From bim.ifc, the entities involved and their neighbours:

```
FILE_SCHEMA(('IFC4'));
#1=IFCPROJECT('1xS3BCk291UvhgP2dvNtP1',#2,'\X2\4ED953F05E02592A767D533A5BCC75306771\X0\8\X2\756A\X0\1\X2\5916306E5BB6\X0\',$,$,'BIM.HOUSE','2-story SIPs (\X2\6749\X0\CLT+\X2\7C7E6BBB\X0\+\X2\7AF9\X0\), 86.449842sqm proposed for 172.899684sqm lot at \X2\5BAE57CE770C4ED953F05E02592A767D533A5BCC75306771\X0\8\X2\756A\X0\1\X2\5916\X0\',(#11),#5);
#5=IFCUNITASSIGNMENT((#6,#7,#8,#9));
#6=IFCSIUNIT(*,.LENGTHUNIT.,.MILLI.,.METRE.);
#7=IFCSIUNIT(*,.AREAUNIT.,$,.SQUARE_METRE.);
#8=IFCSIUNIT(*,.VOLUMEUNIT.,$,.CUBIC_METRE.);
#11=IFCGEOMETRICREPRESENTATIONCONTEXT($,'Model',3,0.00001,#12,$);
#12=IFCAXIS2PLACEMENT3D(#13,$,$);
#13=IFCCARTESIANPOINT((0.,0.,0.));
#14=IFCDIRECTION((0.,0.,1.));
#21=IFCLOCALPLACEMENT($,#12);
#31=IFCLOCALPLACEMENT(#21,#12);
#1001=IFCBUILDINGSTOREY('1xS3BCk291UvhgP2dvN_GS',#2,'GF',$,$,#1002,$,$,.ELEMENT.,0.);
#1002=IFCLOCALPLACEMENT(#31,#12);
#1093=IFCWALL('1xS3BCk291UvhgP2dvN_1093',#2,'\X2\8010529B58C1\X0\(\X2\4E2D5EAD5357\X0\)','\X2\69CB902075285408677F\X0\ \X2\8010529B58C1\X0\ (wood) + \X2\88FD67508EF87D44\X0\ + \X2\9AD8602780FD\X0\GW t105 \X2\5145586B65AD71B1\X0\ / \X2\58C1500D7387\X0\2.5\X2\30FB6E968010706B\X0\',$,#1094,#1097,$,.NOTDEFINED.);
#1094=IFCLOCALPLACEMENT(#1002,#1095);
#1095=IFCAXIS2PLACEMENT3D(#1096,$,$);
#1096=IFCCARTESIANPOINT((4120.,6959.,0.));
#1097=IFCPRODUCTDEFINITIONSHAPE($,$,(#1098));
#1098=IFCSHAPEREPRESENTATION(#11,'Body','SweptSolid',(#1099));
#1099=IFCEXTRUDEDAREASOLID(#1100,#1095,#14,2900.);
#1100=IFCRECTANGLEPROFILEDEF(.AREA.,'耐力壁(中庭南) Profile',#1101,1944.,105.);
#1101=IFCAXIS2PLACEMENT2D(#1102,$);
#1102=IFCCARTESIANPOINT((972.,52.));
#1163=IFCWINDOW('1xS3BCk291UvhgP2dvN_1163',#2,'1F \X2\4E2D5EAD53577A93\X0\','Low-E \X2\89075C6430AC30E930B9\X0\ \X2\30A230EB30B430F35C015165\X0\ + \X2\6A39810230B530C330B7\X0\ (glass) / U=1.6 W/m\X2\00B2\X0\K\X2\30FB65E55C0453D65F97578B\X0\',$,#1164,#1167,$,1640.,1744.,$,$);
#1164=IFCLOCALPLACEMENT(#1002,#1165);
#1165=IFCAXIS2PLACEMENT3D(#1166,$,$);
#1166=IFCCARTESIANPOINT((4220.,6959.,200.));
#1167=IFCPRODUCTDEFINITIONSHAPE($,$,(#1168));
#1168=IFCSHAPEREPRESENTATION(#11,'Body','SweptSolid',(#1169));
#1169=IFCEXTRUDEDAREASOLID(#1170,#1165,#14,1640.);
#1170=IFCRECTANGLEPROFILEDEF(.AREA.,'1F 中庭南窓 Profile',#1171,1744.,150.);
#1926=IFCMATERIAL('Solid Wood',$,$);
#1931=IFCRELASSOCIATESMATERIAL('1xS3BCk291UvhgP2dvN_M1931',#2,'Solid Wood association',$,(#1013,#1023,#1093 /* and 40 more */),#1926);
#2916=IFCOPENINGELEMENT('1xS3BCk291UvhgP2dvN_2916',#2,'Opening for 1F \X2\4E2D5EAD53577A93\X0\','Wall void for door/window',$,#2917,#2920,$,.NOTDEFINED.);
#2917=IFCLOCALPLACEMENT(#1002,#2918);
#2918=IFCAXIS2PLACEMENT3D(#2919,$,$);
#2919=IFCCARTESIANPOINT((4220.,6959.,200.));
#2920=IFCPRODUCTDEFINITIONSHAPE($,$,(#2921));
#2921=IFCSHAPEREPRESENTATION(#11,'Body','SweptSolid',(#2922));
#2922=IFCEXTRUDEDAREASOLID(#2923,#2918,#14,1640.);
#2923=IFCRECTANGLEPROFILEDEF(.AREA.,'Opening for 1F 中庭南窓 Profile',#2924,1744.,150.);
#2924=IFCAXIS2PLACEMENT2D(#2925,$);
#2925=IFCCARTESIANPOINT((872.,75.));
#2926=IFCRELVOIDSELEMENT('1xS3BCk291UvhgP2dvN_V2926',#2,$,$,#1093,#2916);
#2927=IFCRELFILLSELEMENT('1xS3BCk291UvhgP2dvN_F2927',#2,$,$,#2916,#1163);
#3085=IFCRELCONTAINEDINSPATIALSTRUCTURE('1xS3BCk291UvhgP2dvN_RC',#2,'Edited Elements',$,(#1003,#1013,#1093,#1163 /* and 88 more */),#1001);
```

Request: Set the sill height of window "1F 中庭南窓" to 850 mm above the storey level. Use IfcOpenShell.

```python
import numpy as np
import ifcopenshell
import ifcopenshell.api.geometry
import ifcopenshell.geom
import ifcopenshell.util.element
import ifcopenshell.util.placement
import ifcopenshell.util.shape
import ifcopenshell.util.unit

model = ifcopenshell.open("bim.ifc")
unit_scale = ifcopenshell.util.unit.calculate_unit_scale(model)

window = model.by_id(1163)
opening = window.FillsVoids[0].RelatingOpeningElement
storey = ifcopenshell.util.element.get_container(window, ifc_class="IfcBuildingStorey")
level = ifcopenshell.util.placement.get_local_placement(storey.ObjectPlacement)[2, 3]

# The opening's origin need not be at the sill, so measure its lowest point.
shape = ifcopenshell.geom.create_shape(ifcopenshell.geom.settings(), opening)
bottom = ifcopenshell.util.shape.get_shape_bottom_elevation(shape, shape.geometry) / unit_scale
dz = level + 850.0 - bottom

shift = np.array([0.0, 0.0, dz])
# The window is not placed relative to its opening, so move both.
for product in (opening, window):
    matrix = ifcopenshell.util.placement.get_local_placement(product.ObjectPlacement)
    matrix[:3, 3] += shift
    ifcopenshell.api.geometry.edit_object_placement(model, product=product, matrix=matrix, is_si=False)

print(f"moved by {dz * unit_scale:+.3f} m")

model.write("bim_edited.ifc")
```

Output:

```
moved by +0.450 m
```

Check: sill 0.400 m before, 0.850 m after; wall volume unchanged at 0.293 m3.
